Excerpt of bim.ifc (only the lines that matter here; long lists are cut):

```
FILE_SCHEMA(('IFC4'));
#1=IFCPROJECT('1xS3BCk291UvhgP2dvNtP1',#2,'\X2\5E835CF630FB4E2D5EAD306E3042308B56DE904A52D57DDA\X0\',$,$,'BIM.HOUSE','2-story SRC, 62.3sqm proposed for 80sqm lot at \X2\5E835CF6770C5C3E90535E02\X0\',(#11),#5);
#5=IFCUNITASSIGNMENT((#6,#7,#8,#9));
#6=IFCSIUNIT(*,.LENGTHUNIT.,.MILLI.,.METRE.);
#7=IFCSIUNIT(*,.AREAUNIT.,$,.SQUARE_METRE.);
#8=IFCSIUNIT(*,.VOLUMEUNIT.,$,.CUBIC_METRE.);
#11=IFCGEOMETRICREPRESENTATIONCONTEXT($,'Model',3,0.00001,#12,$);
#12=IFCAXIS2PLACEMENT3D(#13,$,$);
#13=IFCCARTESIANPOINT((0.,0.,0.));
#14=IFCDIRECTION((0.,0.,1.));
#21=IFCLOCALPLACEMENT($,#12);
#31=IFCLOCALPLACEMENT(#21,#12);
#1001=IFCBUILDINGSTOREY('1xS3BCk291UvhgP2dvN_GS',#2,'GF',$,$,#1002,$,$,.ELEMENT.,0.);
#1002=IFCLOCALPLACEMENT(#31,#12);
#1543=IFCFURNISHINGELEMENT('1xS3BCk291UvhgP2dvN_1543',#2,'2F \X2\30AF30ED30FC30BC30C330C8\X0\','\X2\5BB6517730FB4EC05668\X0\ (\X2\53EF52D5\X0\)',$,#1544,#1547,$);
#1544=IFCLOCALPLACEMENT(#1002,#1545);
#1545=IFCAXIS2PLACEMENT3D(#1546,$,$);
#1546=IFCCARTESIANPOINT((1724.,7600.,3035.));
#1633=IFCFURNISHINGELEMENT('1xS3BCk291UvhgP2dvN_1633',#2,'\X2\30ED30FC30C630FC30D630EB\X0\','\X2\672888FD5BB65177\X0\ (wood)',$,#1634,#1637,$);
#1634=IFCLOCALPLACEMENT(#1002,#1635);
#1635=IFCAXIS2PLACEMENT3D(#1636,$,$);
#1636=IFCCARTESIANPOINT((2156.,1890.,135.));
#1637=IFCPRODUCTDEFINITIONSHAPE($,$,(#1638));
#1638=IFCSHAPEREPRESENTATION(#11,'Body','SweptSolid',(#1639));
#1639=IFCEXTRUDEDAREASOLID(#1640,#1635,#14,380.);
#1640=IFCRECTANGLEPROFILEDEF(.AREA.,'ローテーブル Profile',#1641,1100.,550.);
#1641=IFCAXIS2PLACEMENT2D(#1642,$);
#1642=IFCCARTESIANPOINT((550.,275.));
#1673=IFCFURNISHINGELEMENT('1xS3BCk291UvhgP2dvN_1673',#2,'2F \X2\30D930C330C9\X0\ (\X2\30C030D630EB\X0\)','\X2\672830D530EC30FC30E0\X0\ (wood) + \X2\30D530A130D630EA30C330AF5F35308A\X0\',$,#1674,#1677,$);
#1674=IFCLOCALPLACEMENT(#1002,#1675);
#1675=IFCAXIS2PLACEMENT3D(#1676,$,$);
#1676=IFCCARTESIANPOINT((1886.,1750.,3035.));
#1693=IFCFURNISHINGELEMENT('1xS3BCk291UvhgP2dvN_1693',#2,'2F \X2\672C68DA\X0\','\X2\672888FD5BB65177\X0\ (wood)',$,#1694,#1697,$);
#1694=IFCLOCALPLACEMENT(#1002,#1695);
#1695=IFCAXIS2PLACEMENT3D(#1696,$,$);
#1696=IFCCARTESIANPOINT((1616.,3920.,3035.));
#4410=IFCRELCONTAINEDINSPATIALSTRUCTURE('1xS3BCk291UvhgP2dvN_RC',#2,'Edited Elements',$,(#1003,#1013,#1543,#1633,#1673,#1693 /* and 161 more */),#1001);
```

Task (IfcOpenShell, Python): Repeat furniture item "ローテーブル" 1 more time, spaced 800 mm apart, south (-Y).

```python
import numpy as np
import ifcopenshell
import ifcopenshell.api.geometry
import ifcopenshell.api.root
import ifcopenshell.util.element
import ifcopenshell.util.placement
import ifcopenshell.util.unit

model = ifcopenshell.open("bim.ifc")
unit_scale = ifcopenshell.util.unit.calculate_unit_scale(model)


def reuse_history(source, copy):
    """copy_class also copies each property set's owner history, people and application; keep the originals."""
    for rel in copy.IsDefinedBy:
        if rel.is_a("IfcRelDefinesByProperties") and (history := rel.RelatingPropertyDefinition.OwnerHistory):
            rel.RelatingPropertyDefinition.OwnerHistory = source.OwnerHistory
            ifcopenshell.util.element.remove_deep2(model, history)


source = model.by_id(1633)
base = ifcopenshell.util.placement.get_local_placement(source.ObjectPlacement)
step = np.array([0.0, -1.0, 0.0]) * 0.8 / unit_scale

for i in range(1, 2):
    copy = ifcopenshell.api.root.copy_class(model, product=source)
    copy.Representation = ifcopenshell.util.element.copy_deep(
        model, source.Representation, exclude=["IfcGeometricRepresentationContext", "IfcRepresentationMap"]
    )
    reuse_history(source, copy)
    matrix = base.copy()
    matrix[:3, 3] += i * step
    print("added at", matrix[:3, 3].round(3) + 0.0)
    ifcopenshell.api.geometry.edit_object_placement(model, product=copy, matrix=matrix, is_si=False)

model.write("bim_edited.ifc")
```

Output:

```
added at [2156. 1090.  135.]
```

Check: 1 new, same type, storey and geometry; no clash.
